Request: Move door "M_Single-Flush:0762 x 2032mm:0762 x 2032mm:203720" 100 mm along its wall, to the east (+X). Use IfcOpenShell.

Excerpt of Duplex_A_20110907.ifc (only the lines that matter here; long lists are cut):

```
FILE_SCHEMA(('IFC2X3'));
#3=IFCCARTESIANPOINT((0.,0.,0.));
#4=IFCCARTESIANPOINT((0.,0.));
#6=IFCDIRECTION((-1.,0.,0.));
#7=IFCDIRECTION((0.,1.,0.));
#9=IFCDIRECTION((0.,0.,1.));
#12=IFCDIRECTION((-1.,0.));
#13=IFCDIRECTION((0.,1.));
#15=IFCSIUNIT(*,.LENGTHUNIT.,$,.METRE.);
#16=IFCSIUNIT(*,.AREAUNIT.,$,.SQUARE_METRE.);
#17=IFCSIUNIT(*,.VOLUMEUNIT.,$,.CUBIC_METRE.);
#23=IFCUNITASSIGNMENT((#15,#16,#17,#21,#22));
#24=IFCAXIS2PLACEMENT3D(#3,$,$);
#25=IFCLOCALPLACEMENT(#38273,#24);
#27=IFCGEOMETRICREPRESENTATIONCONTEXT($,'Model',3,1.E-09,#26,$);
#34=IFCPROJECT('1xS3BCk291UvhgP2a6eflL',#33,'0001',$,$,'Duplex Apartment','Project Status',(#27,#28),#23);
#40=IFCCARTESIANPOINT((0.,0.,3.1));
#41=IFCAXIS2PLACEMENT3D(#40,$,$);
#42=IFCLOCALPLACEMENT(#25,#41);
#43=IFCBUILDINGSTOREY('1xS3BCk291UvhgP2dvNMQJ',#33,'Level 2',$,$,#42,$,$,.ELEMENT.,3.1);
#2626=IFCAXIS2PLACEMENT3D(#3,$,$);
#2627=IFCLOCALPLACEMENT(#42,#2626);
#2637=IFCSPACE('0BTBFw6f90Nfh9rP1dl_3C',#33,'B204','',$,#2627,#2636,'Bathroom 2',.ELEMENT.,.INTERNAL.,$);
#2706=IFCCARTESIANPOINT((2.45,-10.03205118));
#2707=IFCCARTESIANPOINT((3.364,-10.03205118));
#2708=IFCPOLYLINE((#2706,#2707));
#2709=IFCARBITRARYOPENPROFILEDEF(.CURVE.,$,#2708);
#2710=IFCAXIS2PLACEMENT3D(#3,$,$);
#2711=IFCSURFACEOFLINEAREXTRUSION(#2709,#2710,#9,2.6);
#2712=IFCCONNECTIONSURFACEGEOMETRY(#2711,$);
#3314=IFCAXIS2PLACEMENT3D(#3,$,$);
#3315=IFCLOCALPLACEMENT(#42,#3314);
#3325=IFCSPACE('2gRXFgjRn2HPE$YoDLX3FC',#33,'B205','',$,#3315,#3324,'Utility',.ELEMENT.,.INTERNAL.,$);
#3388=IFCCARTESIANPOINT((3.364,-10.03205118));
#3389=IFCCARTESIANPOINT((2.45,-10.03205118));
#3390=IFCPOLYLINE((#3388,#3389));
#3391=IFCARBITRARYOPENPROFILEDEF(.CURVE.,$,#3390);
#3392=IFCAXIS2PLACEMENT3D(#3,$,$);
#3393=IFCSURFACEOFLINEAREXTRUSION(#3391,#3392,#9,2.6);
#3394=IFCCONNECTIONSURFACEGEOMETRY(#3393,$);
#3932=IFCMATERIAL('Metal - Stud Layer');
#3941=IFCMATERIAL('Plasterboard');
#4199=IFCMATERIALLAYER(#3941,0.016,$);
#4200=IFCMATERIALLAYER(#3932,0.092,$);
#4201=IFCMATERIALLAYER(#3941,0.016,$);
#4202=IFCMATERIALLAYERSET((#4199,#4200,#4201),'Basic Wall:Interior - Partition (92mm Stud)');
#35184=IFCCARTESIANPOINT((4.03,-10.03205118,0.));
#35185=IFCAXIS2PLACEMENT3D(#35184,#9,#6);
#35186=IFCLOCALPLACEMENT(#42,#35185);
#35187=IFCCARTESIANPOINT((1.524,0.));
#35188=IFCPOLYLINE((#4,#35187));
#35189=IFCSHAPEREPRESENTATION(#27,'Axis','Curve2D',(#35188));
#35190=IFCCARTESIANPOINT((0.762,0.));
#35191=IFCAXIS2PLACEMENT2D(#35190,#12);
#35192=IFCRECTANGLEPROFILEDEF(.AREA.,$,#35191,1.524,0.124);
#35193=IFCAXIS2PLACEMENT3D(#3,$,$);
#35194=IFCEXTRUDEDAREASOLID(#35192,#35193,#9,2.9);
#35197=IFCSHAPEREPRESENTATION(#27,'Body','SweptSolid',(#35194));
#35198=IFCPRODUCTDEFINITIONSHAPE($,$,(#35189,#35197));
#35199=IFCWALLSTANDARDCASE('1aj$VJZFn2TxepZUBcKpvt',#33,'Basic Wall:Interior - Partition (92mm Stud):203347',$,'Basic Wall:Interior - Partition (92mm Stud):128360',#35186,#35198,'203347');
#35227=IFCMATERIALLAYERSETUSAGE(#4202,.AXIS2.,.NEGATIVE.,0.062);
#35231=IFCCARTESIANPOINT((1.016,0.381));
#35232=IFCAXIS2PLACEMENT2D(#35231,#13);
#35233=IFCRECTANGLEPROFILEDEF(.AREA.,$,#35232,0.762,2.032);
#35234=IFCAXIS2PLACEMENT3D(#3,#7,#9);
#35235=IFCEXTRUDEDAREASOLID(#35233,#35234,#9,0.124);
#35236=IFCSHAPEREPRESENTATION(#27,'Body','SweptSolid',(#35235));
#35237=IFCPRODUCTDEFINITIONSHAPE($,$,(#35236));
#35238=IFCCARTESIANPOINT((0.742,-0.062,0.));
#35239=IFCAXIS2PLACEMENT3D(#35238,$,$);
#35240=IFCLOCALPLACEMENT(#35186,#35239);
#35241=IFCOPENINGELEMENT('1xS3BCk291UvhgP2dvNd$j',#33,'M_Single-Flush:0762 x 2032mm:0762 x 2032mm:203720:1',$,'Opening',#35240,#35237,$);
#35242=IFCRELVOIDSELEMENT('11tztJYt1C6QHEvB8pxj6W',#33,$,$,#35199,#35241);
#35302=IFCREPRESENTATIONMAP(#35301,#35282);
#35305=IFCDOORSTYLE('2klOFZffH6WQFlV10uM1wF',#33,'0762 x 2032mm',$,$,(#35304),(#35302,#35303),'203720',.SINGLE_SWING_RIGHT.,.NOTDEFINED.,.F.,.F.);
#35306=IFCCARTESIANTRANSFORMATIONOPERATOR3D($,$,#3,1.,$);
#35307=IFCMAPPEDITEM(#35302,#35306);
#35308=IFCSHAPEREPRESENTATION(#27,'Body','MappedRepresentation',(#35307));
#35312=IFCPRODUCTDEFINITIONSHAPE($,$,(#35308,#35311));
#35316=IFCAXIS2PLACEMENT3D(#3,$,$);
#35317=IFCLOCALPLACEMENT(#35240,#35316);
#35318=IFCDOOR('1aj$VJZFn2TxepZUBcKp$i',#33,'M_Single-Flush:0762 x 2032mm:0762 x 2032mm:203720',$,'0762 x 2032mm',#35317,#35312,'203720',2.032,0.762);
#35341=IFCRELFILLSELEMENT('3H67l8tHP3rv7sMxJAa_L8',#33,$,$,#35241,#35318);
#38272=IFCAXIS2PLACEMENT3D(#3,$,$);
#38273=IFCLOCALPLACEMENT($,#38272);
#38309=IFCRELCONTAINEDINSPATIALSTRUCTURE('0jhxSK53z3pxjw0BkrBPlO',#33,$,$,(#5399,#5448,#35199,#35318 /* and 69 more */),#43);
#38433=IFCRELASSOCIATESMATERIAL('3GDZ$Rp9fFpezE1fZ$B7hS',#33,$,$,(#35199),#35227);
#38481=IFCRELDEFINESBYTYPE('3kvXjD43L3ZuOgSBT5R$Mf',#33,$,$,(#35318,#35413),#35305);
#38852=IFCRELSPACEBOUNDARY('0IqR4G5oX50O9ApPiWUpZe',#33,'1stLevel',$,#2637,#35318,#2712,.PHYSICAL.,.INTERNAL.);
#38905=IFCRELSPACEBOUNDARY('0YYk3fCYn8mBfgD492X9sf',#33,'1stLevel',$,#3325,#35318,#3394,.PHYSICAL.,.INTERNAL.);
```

```python
import numpy as np
import ifcopenshell
import ifcopenshell.api.geometry
import ifcopenshell.util.placement

model = ifcopenshell.open("Duplex_A_20110907.ifc")

door = model.by_guid("1aj$VJZFn2TxepZUBcKp$i")
opening = door.FillsVoids[0].RelatingOpeningElement
wall = opening.VoidsElements[0].RelatingBuildingElement

wall_matrix = ifcopenshell.util.placement.get_local_placement(wall.ObjectPlacement)
shift = wall_matrix[:3, 0] * -0.1
before = ifcopenshell.util.placement.get_local_placement(door.ObjectPlacement)[:3, 3].copy()

# The door is placed relative to its opening, so it follows when the opening moves.
matrix = ifcopenshell.util.placement.get_local_placement(opening.ObjectPlacement)
matrix[:3, 3] += shift
ifcopenshell.api.geometry.edit_object_placement(
    model, product=opening, matrix=matrix, is_si=False, should_transform_children=True
)

# Space boundary surfaces are stored in each space's coordinates; move them too.
for rel in door.ProvidesBoundaries:
    if not rel.ConnectionGeometry:
        continue
    surface = rel.ConnectionGeometry.SurfaceOnRelatingElement
    space_matrix = ifcopenshell.util.placement.get_local_placement(rel.RelatingSpace.ObjectPlacement)
    point = np.array(surface.Position.Location.Coordinates) + space_matrix[:3, :3].T @ shift
    surface.Position = model.createIfcAxis2Placement3D(
        model.createIfcCartesianPoint(point.tolist()), surface.Position.Axis, surface.Position.RefDirection
    )

after = ifcopenshell.util.placement.get_local_placement(door.ObjectPlacement)[:3, 3]
print("door moved by", (after - before).round(3) + 0.0)

model.write("Duplex_A_20110907_rev.ifc")
```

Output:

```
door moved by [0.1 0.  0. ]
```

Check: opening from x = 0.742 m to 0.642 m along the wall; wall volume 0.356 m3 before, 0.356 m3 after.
